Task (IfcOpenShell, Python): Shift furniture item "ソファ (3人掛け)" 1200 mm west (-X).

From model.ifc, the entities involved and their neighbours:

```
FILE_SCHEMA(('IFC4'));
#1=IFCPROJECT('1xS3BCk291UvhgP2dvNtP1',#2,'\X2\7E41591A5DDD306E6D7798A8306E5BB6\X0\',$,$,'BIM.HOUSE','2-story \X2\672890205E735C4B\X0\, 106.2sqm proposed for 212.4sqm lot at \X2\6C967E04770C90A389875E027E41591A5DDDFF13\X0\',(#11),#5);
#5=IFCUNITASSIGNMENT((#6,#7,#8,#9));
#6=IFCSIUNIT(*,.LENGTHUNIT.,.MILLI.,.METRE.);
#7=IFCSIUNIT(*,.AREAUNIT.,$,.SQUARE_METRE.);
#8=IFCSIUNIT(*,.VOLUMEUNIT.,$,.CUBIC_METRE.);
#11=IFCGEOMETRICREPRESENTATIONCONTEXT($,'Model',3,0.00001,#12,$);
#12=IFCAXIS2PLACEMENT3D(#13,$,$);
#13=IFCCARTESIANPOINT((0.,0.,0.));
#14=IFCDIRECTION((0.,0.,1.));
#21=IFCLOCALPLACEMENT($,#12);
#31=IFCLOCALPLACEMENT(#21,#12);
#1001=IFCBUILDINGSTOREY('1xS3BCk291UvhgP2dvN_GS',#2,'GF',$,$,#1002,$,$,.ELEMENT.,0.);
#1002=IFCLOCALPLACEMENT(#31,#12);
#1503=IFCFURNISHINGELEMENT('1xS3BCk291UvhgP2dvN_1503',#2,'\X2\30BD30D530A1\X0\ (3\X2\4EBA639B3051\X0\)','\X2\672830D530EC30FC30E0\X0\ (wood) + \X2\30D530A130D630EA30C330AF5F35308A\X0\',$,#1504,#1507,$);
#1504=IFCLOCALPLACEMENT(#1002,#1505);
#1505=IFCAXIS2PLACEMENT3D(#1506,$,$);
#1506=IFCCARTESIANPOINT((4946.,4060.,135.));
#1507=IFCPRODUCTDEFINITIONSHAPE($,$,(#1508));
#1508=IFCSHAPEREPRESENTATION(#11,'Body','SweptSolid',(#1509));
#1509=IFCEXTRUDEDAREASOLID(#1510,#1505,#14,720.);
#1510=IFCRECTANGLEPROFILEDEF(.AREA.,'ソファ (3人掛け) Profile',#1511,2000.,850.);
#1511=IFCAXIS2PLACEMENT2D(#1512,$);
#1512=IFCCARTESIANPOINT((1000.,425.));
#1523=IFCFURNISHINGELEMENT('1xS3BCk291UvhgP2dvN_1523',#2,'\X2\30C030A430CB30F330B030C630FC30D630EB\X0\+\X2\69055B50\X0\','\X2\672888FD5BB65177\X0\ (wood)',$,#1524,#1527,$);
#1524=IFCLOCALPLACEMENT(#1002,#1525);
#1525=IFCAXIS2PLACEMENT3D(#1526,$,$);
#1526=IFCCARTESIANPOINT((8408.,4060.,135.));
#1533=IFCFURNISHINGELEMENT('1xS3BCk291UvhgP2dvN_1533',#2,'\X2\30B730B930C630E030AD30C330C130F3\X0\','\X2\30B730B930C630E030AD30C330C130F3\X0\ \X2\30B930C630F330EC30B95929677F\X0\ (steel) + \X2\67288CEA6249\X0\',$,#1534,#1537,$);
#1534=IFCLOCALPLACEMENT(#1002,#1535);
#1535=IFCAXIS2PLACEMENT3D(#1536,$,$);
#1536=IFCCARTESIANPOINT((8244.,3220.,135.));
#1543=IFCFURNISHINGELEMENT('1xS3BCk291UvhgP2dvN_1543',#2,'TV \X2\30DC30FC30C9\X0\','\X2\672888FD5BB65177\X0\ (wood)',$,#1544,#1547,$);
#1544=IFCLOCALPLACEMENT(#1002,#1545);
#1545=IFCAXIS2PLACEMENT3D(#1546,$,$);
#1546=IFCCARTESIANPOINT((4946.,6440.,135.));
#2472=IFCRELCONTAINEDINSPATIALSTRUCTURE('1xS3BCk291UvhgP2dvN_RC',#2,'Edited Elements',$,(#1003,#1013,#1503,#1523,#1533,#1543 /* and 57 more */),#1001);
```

```python
import ifcopenshell
import ifcopenshell.api.geometry
import ifcopenshell.util.placement
import ifcopenshell.util.unit

model = ifcopenshell.open("model.ifc")
unit_scale = ifcopenshell.util.unit.calculate_unit_scale(model)

item = model.by_guid("1xS3BCk291UvhgP2dvN_1503")
matrix = ifcopenshell.util.placement.get_local_placement(item.ObjectPlacement)
matrix[0, 3] -= 1.2 / unit_scale
ifcopenshell.api.geometry.edit_object_placement(model, product=item, matrix=matrix, is_si=False)

print(ifcopenshell.util.placement.get_local_placement(item.ObjectPlacement).round(3) + 0.0)

model.write("model_v2.ifc")
```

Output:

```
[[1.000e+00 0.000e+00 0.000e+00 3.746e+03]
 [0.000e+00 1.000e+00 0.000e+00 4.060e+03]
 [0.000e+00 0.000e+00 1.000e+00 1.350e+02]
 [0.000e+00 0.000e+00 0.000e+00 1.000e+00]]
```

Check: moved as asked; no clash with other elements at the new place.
